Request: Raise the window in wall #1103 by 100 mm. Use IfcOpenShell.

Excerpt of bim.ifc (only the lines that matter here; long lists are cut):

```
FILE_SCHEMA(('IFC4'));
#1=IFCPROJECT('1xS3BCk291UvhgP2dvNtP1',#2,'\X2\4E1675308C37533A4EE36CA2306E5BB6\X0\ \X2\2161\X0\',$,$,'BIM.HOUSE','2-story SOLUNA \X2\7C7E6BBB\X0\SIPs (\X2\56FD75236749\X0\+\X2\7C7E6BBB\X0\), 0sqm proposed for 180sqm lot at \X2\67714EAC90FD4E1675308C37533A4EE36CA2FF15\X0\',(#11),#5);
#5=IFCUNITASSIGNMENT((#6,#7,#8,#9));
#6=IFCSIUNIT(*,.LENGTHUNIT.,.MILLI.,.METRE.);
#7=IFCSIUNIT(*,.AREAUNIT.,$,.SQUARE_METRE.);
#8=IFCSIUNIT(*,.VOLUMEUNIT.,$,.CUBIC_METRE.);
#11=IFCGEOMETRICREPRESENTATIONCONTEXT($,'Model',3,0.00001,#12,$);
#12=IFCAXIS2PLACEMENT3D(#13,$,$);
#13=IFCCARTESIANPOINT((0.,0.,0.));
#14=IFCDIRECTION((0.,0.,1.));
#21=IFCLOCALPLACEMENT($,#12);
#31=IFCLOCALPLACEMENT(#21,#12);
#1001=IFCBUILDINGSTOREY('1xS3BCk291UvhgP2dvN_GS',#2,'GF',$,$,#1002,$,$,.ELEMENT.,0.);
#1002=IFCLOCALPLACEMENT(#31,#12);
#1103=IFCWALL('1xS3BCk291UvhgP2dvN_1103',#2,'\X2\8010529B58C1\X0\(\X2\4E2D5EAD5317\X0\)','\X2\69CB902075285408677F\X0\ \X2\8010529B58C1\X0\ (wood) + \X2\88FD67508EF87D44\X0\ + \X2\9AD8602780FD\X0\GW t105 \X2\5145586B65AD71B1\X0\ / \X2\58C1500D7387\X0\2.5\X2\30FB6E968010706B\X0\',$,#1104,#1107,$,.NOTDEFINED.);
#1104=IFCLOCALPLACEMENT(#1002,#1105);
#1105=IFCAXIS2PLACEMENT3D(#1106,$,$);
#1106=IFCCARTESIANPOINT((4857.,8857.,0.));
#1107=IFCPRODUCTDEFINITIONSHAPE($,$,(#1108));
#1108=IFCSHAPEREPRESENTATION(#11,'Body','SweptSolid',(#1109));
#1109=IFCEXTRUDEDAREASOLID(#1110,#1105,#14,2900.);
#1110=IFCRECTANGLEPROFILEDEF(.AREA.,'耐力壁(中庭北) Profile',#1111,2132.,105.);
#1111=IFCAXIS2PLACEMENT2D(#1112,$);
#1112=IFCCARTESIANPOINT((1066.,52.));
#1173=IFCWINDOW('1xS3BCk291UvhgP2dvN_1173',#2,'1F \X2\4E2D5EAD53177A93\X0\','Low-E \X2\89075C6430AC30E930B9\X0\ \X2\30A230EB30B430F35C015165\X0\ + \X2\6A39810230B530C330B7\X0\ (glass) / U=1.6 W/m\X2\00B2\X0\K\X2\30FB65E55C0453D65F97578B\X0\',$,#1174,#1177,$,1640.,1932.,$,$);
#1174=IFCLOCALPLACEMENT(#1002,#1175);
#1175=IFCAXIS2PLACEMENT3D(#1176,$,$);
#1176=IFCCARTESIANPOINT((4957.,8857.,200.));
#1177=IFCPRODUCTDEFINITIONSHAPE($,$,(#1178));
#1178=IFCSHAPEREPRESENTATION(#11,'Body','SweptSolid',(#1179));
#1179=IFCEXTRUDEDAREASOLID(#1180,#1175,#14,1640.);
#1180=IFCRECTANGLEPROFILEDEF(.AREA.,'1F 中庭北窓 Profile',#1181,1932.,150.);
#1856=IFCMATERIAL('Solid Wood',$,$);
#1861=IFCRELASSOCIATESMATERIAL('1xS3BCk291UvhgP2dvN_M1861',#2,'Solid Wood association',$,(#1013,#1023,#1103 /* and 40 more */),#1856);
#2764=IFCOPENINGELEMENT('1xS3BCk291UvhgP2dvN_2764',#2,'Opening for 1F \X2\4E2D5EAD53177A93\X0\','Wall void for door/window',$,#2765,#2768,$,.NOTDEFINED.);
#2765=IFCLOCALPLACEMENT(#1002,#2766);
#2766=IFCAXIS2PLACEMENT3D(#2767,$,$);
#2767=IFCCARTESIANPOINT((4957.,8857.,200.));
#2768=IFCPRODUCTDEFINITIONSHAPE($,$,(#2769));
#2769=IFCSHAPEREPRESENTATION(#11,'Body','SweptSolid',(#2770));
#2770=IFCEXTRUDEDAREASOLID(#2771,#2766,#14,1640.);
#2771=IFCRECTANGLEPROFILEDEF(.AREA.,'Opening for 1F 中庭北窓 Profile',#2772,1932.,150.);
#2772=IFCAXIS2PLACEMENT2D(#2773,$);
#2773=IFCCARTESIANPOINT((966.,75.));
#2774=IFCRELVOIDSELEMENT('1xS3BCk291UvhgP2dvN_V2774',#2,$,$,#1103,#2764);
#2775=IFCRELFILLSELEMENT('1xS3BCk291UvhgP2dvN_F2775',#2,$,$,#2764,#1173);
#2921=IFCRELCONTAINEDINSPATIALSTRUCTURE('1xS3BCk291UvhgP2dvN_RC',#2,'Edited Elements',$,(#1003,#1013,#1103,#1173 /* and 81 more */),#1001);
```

```python
import numpy as np
import ifcopenshell
import ifcopenshell.api.geometry
import ifcopenshell.util.placement
import ifcopenshell.util.unit

model = ifcopenshell.open("bim.ifc")
unit_scale = ifcopenshell.util.unit.calculate_unit_scale(model)

window = model.by_guid("1xS3BCk291UvhgP2dvN_1173")
opening = window.FillsVoids[0].RelatingOpeningElement
dz = 0.1 / unit_scale

shift = np.array([0.0, 0.0, dz])
# The window is not placed relative to its opening, so move both.
for product in (opening, window):
    matrix = ifcopenshell.util.placement.get_local_placement(product.ObjectPlacement)
    matrix[:3, 3] += shift
    ifcopenshell.api.geometry.edit_object_placement(model, product=product, matrix=matrix, is_si=False)

print(f"moved by {dz * unit_scale:+.3f} m")

model.write("bim_updated.ifc")
```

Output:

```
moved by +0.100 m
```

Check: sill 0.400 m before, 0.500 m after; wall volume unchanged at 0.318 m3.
